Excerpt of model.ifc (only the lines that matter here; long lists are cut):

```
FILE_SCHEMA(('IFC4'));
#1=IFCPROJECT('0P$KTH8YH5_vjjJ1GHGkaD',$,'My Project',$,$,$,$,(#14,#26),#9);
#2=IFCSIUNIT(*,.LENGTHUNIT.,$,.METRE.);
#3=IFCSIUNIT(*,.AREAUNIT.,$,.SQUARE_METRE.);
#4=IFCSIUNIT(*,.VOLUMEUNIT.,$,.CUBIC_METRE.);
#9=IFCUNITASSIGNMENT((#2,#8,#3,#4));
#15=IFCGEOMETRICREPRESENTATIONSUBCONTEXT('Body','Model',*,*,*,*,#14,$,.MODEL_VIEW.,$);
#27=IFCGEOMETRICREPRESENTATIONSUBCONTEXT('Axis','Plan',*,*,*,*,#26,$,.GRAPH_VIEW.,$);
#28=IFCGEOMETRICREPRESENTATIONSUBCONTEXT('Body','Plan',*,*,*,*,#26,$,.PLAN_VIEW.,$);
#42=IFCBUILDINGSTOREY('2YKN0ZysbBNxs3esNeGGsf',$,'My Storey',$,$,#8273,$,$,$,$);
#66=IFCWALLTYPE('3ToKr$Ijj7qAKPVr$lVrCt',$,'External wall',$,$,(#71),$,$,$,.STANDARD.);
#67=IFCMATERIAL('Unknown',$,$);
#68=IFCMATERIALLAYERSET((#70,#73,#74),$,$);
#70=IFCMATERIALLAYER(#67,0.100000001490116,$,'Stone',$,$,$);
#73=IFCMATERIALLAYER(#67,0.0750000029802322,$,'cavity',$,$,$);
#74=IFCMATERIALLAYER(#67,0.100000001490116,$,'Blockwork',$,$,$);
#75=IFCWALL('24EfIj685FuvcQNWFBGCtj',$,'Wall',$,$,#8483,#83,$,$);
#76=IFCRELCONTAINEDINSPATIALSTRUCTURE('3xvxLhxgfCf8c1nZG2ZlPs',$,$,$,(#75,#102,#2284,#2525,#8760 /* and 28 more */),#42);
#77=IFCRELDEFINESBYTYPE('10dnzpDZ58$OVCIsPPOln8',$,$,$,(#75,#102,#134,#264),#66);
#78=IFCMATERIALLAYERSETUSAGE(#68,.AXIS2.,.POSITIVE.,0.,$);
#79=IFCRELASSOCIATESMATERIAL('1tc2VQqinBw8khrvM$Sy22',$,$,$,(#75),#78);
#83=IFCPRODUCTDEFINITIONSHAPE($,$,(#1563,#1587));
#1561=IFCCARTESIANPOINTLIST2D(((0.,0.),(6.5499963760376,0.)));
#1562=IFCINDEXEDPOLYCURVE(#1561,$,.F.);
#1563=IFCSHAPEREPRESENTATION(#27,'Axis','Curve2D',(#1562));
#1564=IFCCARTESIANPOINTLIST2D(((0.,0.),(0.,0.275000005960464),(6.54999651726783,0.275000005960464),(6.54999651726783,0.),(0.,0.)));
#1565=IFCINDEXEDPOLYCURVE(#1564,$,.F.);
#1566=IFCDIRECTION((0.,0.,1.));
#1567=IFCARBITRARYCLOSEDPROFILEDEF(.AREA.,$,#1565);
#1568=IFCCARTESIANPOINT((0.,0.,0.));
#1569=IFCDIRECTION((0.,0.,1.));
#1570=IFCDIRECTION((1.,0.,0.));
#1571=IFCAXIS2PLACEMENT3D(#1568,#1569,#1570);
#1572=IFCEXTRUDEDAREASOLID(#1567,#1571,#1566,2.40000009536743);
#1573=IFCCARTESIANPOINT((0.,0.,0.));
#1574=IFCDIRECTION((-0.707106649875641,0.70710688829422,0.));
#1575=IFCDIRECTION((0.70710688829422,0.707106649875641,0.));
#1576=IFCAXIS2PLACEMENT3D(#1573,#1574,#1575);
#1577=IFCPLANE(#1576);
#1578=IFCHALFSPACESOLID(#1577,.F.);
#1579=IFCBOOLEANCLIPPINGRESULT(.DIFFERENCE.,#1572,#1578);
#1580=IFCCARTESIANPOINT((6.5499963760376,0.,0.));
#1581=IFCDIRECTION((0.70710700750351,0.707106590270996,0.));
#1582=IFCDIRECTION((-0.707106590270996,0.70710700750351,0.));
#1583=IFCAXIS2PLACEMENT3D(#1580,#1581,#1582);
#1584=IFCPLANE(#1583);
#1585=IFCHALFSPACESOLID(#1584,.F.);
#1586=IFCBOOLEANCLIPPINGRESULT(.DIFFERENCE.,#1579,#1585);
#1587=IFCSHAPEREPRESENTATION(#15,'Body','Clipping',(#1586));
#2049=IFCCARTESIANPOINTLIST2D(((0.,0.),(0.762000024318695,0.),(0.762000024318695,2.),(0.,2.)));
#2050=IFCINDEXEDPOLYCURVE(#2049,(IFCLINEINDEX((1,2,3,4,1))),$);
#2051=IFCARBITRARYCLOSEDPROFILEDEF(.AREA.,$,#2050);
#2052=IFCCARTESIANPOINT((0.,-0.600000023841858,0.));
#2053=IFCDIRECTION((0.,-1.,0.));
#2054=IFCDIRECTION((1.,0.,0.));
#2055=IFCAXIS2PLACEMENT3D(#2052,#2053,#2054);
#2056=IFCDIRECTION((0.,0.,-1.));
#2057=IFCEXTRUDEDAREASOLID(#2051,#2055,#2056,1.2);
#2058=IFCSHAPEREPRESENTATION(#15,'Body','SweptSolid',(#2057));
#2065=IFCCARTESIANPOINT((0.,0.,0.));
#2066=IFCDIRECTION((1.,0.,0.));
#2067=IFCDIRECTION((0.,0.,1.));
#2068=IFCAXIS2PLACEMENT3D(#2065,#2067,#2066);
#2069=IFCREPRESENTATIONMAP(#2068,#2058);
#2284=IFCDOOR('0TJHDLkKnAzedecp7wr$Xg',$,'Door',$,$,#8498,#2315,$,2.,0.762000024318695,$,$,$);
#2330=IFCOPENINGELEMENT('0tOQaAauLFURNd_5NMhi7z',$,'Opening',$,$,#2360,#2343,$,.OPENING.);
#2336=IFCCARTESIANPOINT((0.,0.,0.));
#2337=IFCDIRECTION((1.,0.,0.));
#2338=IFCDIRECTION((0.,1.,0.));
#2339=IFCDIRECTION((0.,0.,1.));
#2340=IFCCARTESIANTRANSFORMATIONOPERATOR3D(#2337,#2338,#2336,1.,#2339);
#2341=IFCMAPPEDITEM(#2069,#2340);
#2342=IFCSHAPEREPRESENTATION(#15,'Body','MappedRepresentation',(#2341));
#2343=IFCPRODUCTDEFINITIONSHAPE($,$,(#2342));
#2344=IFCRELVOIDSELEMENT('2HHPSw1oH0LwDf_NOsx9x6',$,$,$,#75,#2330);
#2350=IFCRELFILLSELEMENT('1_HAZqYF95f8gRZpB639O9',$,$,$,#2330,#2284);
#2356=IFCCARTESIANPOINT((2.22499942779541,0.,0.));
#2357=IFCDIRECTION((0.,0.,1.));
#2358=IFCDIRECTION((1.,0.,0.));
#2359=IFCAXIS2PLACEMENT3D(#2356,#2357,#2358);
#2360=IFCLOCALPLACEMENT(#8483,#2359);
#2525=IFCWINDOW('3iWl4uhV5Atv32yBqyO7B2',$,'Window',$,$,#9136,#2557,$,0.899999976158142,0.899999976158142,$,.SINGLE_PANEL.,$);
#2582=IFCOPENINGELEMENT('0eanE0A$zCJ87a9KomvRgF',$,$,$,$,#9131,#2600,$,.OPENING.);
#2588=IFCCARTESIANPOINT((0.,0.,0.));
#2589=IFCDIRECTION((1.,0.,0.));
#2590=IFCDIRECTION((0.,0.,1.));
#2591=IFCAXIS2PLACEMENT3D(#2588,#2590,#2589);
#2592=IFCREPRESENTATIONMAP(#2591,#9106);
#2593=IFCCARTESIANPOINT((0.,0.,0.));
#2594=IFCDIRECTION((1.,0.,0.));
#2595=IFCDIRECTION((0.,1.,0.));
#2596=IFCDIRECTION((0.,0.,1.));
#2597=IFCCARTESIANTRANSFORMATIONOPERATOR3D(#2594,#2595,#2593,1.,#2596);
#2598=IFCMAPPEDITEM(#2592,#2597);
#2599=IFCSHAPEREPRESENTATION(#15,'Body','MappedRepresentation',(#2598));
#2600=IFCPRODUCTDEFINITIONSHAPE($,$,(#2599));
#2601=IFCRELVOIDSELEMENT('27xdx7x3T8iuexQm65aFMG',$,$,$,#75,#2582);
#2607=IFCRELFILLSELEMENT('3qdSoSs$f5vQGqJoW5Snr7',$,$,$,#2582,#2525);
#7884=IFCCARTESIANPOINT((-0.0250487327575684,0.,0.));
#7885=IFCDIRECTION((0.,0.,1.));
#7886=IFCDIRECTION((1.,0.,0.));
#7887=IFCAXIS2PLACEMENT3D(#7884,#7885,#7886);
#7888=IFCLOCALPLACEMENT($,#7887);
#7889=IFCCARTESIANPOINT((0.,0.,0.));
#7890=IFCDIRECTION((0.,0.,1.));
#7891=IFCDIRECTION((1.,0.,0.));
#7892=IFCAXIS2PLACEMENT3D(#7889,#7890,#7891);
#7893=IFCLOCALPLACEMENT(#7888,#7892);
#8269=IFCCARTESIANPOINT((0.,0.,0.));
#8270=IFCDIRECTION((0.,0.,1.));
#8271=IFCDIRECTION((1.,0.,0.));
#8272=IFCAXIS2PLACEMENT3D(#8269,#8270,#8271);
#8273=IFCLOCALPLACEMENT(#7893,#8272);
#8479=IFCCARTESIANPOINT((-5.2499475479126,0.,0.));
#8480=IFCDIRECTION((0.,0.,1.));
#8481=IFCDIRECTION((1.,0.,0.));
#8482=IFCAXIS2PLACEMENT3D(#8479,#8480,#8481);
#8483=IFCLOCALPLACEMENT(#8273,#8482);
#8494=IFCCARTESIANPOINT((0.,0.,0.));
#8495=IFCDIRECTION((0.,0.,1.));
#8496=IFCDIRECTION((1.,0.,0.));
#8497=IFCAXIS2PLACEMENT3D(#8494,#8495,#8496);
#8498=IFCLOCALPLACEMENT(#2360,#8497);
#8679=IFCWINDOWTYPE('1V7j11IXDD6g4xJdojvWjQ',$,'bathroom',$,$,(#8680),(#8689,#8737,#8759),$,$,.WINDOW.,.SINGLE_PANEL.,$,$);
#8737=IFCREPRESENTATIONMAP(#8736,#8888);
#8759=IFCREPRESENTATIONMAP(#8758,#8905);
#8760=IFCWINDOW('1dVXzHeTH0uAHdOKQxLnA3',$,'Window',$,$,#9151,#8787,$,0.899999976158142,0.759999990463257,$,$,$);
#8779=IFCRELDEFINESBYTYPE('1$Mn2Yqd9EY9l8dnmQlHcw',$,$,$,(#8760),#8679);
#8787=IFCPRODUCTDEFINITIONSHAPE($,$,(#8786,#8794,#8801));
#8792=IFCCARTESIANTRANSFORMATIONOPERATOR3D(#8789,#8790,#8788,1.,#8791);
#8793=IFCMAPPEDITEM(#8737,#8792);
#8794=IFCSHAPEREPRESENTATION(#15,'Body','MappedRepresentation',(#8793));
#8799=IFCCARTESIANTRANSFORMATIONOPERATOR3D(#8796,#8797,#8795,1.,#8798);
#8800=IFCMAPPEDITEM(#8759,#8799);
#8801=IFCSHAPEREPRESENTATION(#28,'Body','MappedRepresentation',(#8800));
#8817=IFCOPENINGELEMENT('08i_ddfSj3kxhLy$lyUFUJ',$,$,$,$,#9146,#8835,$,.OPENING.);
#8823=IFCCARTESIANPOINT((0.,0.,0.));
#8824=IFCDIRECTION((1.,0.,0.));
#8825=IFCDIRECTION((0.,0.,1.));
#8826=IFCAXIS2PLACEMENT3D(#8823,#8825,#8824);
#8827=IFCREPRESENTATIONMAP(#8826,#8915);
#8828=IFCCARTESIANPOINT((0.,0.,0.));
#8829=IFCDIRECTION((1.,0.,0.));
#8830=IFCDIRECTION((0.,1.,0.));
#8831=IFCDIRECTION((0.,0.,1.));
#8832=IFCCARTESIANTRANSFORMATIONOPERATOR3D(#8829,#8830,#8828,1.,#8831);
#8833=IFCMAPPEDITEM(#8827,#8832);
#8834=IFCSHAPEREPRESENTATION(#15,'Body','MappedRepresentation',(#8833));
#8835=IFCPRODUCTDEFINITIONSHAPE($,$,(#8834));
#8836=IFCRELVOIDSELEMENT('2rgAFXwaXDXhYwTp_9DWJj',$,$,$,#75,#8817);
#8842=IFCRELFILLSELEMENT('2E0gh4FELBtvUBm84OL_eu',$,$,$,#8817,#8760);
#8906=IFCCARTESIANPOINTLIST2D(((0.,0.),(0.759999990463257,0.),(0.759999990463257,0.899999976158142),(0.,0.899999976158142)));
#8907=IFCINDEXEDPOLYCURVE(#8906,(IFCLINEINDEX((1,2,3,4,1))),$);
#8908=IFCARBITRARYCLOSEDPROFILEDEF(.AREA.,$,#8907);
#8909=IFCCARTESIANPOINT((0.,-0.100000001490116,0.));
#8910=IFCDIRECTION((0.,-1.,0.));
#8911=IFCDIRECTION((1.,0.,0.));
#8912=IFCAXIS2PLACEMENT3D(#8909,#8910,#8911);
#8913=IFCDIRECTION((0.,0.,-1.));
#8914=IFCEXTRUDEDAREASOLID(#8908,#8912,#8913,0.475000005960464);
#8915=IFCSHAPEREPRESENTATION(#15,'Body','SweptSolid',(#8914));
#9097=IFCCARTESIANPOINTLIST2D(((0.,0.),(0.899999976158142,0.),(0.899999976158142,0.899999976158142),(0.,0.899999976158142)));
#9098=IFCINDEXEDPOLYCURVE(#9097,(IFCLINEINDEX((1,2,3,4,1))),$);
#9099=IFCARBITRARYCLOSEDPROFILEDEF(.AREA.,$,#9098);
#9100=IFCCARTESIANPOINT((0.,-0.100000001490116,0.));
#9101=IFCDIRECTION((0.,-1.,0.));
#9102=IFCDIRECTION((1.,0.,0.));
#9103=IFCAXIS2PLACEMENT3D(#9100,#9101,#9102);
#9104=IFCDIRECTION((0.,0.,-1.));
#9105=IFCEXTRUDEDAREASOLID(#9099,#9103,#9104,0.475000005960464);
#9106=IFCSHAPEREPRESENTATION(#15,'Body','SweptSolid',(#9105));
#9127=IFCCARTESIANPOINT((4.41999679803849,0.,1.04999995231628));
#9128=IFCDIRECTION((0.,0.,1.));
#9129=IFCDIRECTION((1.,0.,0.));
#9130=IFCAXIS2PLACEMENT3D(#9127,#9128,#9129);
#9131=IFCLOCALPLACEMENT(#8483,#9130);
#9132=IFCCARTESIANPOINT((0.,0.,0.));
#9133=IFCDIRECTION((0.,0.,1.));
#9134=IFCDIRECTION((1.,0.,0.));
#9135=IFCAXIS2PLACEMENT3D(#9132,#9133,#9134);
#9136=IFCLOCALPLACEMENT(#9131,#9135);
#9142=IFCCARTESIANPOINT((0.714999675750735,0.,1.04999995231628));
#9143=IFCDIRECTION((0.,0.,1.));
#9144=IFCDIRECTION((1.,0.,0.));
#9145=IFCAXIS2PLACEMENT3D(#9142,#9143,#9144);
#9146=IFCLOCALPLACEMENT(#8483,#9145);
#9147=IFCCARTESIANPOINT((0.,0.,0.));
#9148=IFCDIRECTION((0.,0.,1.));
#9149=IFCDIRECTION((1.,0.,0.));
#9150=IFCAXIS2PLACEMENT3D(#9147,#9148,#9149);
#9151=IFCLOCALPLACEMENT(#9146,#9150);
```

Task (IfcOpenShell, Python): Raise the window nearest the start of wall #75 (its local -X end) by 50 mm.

```python
import numpy as np
import ifcopenshell
import ifcopenshell.api.geometry
import ifcopenshell.util.placement
import ifcopenshell.util.unit

model = ifcopenshell.open("model.ifc")
unit_scale = ifcopenshell.util.unit.calculate_unit_scale(model)

window = model.by_id(8760)
opening = window.FillsVoids[0].RelatingOpeningElement
dz = 0.05 / unit_scale

shift = np.array([0.0, 0.0, dz])
# The window is placed relative to its opening, so it follows when the opening moves.
matrix = ifcopenshell.util.placement.get_local_placement(opening.ObjectPlacement)
matrix[:3, 3] += shift
ifcopenshell.api.geometry.edit_object_placement(
    model, product=opening, matrix=matrix, is_si=False, should_transform_children=True
)

print(f"moved by {dz * unit_scale:+.3f} m")

model.write("model_edited.ifc")
```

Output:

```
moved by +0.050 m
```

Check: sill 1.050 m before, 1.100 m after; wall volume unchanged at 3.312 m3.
